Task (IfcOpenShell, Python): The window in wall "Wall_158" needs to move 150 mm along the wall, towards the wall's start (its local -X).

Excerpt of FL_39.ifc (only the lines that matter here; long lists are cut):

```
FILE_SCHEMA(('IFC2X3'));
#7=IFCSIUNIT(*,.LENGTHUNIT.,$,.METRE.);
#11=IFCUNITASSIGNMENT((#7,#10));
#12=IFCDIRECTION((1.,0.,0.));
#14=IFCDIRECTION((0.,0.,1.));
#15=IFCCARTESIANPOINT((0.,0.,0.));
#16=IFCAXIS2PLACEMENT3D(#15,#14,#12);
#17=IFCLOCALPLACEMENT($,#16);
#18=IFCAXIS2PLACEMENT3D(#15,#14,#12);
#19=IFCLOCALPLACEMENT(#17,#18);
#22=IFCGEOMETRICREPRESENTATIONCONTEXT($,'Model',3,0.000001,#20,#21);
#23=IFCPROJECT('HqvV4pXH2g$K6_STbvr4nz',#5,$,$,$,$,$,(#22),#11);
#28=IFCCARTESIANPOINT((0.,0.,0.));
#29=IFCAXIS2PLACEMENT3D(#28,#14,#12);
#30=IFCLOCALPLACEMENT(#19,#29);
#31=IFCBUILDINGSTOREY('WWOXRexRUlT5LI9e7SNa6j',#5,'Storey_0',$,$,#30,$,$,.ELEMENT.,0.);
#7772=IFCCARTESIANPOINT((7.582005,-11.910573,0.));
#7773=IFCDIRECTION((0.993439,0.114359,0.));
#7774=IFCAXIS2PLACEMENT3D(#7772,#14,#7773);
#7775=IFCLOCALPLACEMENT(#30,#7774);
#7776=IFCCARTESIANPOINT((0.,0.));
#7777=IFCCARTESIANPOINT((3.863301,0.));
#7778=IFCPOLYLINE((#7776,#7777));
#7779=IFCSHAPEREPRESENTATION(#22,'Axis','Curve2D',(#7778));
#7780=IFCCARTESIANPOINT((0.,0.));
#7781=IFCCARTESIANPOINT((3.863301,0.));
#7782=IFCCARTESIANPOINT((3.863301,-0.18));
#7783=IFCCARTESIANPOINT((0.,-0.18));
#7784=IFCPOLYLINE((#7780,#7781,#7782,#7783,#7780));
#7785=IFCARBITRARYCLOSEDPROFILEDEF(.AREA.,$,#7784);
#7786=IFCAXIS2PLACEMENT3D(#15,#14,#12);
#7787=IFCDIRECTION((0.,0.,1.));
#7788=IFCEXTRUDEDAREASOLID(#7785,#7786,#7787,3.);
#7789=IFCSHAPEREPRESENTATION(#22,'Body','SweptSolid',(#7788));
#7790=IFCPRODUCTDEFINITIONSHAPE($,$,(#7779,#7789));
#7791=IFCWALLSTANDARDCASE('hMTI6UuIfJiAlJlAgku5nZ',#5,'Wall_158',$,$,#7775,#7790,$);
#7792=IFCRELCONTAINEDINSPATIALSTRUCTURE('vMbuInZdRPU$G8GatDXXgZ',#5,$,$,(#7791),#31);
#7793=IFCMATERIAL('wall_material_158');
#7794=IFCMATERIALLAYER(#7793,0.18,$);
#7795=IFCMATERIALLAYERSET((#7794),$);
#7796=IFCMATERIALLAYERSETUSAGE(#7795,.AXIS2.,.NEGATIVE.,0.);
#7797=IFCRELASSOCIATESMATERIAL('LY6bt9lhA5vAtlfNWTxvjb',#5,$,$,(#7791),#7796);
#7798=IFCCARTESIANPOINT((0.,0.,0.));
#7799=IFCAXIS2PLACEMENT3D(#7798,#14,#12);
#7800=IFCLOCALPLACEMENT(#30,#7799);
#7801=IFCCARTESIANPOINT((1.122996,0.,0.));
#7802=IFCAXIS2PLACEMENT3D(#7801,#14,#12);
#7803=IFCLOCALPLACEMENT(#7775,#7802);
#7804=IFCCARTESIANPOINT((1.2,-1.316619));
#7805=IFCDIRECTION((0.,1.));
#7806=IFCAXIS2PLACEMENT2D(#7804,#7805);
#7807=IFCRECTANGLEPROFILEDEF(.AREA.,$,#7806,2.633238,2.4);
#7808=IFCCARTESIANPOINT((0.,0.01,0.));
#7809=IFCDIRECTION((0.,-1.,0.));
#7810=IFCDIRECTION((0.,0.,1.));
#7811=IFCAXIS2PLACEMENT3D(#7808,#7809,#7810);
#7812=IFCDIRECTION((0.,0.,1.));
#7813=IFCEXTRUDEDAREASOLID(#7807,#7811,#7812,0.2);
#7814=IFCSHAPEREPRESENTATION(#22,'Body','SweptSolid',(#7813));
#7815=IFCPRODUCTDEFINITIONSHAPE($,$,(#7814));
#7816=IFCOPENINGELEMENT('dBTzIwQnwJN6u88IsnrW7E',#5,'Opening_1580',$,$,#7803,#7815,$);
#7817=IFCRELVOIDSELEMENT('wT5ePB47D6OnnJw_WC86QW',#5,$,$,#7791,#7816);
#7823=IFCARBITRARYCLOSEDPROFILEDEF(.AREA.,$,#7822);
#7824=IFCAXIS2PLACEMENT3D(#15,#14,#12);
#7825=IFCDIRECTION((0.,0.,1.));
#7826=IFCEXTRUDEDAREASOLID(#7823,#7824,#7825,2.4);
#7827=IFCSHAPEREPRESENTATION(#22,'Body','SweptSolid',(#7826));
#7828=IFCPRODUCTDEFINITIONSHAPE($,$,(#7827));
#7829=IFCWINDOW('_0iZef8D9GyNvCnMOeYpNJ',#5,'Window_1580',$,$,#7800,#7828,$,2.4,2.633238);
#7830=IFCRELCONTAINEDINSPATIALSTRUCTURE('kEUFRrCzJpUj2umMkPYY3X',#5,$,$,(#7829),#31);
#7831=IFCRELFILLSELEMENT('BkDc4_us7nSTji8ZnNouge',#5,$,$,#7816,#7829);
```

```python
import ifcopenshell
import ifcopenshell.api.geometry
import ifcopenshell.util.placement
import ifcopenshell.util.unit

model = ifcopenshell.open("FL_39.ifc")
unit_scale = ifcopenshell.util.unit.calculate_unit_scale(model)

window = model.by_id(7829)
opening = window.FillsVoids[0].RelatingOpeningElement
wall = opening.VoidsElements[0].RelatingBuildingElement

wall_matrix = ifcopenshell.util.placement.get_local_placement(wall.ObjectPlacement)
shift = wall_matrix[:3, 0] * -0.15 / unit_scale
before = ifcopenshell.util.placement.get_local_placement(window.ObjectPlacement)[:3, 3].copy()

# The window is not placed relative to its opening, so move both.
for product in (opening, window):
    matrix = ifcopenshell.util.placement.get_local_placement(product.ObjectPlacement)
    matrix[:3, 3] += shift
    ifcopenshell.api.geometry.edit_object_placement(model, product=product, matrix=matrix, is_si=False)

after = ifcopenshell.util.placement.get_local_placement(window.ObjectPlacement)[:3, 3]
print("window moved by", (after - before).round(3) + 0.0)

model.write("FL_39-out.ifc")
```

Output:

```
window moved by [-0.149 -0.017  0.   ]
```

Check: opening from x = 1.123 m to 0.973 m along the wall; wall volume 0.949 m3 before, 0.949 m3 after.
